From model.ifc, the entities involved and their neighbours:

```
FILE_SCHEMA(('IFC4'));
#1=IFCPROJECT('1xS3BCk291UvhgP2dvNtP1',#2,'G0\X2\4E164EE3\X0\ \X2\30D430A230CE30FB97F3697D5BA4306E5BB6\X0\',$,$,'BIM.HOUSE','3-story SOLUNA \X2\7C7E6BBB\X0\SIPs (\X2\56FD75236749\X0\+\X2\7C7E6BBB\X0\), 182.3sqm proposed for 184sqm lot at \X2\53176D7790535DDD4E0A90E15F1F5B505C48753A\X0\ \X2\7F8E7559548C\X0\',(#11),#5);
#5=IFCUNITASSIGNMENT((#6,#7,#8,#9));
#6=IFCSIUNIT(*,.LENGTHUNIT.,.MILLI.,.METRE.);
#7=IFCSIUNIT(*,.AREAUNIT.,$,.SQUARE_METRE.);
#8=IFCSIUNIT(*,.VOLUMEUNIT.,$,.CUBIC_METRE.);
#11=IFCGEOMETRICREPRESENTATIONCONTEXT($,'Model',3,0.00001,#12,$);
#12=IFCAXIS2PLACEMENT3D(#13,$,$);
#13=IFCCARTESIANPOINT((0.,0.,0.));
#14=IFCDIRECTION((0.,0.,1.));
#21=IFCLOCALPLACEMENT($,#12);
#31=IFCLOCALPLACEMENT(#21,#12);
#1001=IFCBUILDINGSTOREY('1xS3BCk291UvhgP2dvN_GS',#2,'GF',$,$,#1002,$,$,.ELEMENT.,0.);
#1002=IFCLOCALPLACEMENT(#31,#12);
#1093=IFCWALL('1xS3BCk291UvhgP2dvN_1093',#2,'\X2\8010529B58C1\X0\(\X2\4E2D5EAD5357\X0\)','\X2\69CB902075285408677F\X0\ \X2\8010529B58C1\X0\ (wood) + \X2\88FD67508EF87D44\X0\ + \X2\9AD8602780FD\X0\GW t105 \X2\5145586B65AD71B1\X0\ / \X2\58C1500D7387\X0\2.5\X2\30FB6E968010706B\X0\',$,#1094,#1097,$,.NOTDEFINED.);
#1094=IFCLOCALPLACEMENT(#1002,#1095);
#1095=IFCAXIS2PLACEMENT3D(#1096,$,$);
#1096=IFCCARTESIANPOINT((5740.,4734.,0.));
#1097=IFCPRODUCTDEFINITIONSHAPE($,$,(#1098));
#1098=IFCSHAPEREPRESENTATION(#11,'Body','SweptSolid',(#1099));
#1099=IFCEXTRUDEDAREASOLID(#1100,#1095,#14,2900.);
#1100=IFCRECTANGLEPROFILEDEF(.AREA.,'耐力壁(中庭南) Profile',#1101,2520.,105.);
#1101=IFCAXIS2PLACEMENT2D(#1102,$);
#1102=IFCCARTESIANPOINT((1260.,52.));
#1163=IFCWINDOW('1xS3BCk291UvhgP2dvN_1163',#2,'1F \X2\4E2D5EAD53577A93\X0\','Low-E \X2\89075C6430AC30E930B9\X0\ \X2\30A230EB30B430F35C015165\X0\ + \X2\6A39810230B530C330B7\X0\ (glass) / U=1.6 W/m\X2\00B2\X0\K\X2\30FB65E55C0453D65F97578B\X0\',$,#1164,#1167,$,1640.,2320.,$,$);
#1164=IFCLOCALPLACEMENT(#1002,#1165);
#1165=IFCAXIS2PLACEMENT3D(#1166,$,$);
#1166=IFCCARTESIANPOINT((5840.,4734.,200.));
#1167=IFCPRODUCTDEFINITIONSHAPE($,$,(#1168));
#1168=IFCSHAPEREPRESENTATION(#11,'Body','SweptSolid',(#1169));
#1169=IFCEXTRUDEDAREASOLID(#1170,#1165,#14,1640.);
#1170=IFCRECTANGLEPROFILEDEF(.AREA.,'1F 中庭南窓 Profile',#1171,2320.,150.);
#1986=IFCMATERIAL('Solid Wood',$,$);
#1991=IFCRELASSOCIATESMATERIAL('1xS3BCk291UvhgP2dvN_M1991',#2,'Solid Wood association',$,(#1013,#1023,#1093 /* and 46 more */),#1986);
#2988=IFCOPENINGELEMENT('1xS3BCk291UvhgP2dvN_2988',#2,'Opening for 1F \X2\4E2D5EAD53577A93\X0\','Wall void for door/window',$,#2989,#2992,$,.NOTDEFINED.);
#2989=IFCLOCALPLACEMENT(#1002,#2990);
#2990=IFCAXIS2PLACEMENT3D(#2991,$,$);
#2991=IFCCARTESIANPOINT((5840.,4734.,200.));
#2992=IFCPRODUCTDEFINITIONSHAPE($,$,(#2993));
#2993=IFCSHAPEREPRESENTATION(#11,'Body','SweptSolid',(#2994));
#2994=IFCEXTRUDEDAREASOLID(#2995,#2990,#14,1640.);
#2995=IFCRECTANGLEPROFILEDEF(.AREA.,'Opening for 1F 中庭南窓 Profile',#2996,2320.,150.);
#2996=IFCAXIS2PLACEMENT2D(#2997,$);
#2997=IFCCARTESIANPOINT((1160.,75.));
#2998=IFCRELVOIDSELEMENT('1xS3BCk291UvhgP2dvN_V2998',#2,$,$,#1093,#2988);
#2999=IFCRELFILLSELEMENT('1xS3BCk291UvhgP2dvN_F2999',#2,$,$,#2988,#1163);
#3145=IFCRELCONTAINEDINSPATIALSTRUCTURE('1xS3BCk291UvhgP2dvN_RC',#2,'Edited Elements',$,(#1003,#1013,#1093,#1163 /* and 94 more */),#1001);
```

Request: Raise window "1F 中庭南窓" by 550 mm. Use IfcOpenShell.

```python
import numpy as np
import ifcopenshell
import ifcopenshell.api.geometry
import ifcopenshell.util.placement
import ifcopenshell.util.unit

model = ifcopenshell.open("model.ifc")
unit_scale = ifcopenshell.util.unit.calculate_unit_scale(model)

window = model.by_guid("1xS3BCk291UvhgP2dvN_1163")
opening = window.FillsVoids[0].RelatingOpeningElement
dz = 0.55 / unit_scale

shift = np.array([0.0, 0.0, dz])
# The window is not placed relative to its opening, so move both.
for product in (opening, window):
    matrix = ifcopenshell.util.placement.get_local_placement(product.ObjectPlacement)
    matrix[:3, 3] += shift
    ifcopenshell.api.geometry.edit_object_placement(model, product=product, matrix=matrix, is_si=False)

print(f"moved by {dz * unit_scale:+.3f} m")

model.write("model_v2.ifc")
```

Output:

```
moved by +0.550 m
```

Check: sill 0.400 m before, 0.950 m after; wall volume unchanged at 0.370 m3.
